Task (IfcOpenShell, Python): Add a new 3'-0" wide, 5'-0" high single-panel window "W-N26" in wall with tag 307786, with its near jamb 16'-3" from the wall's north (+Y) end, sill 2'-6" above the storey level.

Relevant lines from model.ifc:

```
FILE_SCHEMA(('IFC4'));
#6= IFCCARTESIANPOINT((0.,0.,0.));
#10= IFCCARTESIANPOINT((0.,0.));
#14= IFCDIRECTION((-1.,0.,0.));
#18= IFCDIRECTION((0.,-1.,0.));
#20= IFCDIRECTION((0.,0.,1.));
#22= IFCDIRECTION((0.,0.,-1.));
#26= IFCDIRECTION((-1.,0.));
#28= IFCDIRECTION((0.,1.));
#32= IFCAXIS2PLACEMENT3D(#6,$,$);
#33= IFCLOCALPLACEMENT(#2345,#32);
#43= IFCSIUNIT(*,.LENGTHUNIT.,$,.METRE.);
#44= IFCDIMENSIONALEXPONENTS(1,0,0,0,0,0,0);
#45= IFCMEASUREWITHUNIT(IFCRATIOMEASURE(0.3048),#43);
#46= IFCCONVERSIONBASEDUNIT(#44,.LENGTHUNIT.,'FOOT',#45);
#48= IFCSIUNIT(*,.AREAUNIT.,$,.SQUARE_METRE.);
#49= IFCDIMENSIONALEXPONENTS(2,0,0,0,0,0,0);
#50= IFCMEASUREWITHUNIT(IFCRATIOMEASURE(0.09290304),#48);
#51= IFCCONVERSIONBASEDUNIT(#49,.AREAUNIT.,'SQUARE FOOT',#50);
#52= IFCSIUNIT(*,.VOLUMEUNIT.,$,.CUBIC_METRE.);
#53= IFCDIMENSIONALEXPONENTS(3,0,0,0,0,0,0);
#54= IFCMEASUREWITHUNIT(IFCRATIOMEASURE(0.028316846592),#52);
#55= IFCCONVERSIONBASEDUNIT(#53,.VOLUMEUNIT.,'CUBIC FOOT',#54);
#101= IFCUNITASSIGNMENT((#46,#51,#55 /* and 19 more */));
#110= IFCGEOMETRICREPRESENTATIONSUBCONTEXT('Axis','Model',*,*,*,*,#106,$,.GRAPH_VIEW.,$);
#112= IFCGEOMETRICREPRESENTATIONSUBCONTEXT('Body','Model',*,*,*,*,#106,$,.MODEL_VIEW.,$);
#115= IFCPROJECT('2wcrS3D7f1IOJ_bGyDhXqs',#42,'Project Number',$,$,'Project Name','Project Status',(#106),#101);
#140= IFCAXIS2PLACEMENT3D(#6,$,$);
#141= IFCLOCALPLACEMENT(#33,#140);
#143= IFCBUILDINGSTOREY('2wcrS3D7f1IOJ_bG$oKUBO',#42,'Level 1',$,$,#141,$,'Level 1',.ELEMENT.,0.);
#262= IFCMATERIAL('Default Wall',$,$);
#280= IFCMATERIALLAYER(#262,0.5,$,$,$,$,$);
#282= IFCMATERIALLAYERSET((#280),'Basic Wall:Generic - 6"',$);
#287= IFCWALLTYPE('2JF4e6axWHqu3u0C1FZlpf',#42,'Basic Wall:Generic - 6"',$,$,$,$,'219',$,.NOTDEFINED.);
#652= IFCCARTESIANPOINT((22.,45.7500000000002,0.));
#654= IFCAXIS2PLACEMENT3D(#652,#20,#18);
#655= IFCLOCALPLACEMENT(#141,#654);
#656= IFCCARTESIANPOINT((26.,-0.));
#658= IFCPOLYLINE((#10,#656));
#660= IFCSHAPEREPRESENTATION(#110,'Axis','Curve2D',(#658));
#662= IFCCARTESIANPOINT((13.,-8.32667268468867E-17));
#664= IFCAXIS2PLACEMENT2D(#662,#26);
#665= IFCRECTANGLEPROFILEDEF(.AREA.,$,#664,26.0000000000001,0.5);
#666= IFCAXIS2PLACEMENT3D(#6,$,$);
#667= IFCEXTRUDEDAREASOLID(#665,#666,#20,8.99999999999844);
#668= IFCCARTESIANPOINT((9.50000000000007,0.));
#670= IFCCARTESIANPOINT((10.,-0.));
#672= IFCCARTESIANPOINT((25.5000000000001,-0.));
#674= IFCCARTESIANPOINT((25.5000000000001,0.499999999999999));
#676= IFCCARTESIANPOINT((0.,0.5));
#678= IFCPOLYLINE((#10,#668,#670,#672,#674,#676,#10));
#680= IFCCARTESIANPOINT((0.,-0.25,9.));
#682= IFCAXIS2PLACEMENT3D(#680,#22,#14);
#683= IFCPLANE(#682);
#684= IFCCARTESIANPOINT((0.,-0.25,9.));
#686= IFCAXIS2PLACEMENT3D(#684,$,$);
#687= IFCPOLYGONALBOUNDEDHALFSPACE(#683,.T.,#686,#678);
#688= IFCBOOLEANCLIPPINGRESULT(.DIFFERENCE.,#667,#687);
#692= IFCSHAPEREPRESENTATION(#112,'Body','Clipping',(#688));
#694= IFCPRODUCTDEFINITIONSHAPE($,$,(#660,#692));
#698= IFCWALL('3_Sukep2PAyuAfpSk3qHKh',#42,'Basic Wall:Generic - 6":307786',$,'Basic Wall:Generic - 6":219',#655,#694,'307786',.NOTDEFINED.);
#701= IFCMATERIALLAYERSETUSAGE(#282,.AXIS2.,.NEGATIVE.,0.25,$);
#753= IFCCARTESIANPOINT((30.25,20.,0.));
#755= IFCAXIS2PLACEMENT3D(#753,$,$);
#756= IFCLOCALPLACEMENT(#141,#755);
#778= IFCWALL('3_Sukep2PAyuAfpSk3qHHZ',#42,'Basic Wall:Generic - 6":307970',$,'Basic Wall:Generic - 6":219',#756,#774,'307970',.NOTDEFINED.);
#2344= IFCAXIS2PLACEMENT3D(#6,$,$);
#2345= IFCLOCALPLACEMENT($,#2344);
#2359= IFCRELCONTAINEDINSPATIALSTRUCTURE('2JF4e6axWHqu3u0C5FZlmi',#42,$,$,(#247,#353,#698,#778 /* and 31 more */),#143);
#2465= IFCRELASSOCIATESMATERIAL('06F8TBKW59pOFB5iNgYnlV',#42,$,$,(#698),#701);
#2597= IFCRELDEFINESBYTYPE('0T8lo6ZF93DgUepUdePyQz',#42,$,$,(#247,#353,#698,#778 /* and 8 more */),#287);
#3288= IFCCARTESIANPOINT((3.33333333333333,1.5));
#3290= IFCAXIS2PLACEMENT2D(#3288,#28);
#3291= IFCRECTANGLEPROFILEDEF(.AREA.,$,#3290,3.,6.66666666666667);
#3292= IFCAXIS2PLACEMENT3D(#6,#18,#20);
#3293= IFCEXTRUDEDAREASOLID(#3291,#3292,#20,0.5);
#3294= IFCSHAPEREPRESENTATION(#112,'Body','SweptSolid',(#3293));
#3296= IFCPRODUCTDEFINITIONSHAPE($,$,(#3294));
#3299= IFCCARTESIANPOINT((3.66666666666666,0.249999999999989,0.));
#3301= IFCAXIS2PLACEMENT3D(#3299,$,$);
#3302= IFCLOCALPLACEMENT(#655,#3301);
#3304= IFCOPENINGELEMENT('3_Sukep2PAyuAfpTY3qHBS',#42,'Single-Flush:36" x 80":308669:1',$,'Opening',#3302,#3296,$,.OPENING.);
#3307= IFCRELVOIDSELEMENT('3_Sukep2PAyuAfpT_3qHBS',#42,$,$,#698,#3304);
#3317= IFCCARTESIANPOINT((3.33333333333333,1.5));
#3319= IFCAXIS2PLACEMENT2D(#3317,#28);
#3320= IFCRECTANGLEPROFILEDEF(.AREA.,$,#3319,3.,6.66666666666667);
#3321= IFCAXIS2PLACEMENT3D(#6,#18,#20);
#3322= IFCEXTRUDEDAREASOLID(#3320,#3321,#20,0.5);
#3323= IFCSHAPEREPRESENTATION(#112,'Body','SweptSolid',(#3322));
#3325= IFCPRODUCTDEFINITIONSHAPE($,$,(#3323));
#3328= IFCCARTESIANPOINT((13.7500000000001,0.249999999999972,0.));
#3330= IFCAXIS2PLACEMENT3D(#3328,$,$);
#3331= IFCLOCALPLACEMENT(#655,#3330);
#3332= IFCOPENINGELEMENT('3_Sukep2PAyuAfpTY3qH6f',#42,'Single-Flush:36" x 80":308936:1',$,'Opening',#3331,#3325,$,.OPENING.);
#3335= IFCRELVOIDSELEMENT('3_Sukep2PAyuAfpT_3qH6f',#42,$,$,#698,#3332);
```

```python
import numpy as np
import ifcopenshell
import ifcopenshell.api.feature
import ifcopenshell.api.geometry
import ifcopenshell.api.root
import ifcopenshell.api.spatial
import ifcopenshell.geom
import ifcopenshell.util.element
import ifcopenshell.util.placement
import ifcopenshell.util.representation
import ifcopenshell.util.shape
import ifcopenshell.util.unit

model = ifcopenshell.open("model.ifc")
unit_scale = ifcopenshell.util.unit.calculate_unit_scale(model)
settings = ifcopenshell.geom.settings()


def volume(element):
    """Net volume in cubic metres, openings subtracted."""
    shape = ifcopenshell.geom.create_shape(settings, element)
    return ifcopenshell.util.shape.get_volume(shape.geometry)


wall = model.by_id(698)
storey = ifcopenshell.util.element.get_container(wall, ifc_class="IfcBuildingStorey")
context = ifcopenshell.util.representation.get_context(model, "Model", "Body", "MODEL_VIEW")
before = volume(wall)

width, height, from_end, sill = 0.9144, 1.524, 4.953, 0.762  # metres

# The wall runs along its own X axis, and the end named is its -X end.
wall_shape = ifcopenshell.geom.create_shape(settings, wall)
x, y, z = ifcopenshell.util.shape.get_vertices(wall_shape.geometry).T
start = x.min() + from_end
face, thickness = float(y.min()), float(y.max() - y.min())
wall_matrix = ifcopenshell.util.placement.get_local_placement(wall.ObjectPlacement)
level = ifcopenshell.util.placement.get_local_placement(storey.ObjectPlacement)[2, 3]


def in_wall(x, y):
    """Placement at x, y metres in the wall's axes, at sill height."""
    matrix = wall_matrix.copy()
    matrix[:, 3] = wall_matrix @ np.array([x / unit_scale, y / unit_scale, 0.0, 1.0])
    matrix[2, 3] = level + sill / unit_scale
    return matrix


# Opening: a box that overshoots both wall faces by 50 mm.
opening = ifcopenshell.api.root.create_entity(model, ifc_class="IfcOpeningElement", predefined_type="OPENING")
box = ifcopenshell.api.geometry.add_wall_representation(
    model, context=context, length=width, height=height, thickness=thickness + 0.1
)
ifcopenshell.api.geometry.assign_representation(model, product=opening, representation=box)
ifcopenshell.api.geometry.edit_object_placement(model, product=opening, matrix=in_wall(start, face - 0.05), is_si=False)
ifcopenshell.api.feature.add_feature(model, feature=opening, element=wall)

window = ifcopenshell.api.root.create_entity(model, ifc_class="IfcWindow", name="W-N26", predefined_type="WINDOW")
window.OverallWidth, window.OverallHeight = width / unit_scale, height / unit_scale
window.PartitioningType = "SINGLE_PANEL"
body = ifcopenshell.api.geometry.add_window_representation(
    model,
    context=context,
    overall_width=window.OverallWidth,
    overall_height=window.OverallHeight,
    partition_type="SINGLE_PANEL",
)
ifcopenshell.api.geometry.assign_representation(model, product=window, representation=body)
ifcopenshell.api.spatial.assign_container(model, products=[window], relating_structure=storey)
ifcopenshell.api.feature.add_filling(model, opening=opening, element=window)

# Centre the window in the wall's thickness.
ifcopenshell.api.geometry.edit_object_placement(model, product=window, matrix=in_wall(start, face), is_si=False)
window_shape = ifcopenshell.geom.create_shape(settings, window)
depth = ifcopenshell.util.shape.get_vertices(window_shape.geometry)[:, 1]
offset = face + thickness / 2 - (depth.min() + depth.max()) / 2
ifcopenshell.api.geometry.edit_object_placement(model, product=window, matrix=in_wall(start, offset), is_si=False)

after = volume(wall)

print(f"wall volume {before:.3f} -> {after:.3f} m3")

model.write("model_edited.ifc")
```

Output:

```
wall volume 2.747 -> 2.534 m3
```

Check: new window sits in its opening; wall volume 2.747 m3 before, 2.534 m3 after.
